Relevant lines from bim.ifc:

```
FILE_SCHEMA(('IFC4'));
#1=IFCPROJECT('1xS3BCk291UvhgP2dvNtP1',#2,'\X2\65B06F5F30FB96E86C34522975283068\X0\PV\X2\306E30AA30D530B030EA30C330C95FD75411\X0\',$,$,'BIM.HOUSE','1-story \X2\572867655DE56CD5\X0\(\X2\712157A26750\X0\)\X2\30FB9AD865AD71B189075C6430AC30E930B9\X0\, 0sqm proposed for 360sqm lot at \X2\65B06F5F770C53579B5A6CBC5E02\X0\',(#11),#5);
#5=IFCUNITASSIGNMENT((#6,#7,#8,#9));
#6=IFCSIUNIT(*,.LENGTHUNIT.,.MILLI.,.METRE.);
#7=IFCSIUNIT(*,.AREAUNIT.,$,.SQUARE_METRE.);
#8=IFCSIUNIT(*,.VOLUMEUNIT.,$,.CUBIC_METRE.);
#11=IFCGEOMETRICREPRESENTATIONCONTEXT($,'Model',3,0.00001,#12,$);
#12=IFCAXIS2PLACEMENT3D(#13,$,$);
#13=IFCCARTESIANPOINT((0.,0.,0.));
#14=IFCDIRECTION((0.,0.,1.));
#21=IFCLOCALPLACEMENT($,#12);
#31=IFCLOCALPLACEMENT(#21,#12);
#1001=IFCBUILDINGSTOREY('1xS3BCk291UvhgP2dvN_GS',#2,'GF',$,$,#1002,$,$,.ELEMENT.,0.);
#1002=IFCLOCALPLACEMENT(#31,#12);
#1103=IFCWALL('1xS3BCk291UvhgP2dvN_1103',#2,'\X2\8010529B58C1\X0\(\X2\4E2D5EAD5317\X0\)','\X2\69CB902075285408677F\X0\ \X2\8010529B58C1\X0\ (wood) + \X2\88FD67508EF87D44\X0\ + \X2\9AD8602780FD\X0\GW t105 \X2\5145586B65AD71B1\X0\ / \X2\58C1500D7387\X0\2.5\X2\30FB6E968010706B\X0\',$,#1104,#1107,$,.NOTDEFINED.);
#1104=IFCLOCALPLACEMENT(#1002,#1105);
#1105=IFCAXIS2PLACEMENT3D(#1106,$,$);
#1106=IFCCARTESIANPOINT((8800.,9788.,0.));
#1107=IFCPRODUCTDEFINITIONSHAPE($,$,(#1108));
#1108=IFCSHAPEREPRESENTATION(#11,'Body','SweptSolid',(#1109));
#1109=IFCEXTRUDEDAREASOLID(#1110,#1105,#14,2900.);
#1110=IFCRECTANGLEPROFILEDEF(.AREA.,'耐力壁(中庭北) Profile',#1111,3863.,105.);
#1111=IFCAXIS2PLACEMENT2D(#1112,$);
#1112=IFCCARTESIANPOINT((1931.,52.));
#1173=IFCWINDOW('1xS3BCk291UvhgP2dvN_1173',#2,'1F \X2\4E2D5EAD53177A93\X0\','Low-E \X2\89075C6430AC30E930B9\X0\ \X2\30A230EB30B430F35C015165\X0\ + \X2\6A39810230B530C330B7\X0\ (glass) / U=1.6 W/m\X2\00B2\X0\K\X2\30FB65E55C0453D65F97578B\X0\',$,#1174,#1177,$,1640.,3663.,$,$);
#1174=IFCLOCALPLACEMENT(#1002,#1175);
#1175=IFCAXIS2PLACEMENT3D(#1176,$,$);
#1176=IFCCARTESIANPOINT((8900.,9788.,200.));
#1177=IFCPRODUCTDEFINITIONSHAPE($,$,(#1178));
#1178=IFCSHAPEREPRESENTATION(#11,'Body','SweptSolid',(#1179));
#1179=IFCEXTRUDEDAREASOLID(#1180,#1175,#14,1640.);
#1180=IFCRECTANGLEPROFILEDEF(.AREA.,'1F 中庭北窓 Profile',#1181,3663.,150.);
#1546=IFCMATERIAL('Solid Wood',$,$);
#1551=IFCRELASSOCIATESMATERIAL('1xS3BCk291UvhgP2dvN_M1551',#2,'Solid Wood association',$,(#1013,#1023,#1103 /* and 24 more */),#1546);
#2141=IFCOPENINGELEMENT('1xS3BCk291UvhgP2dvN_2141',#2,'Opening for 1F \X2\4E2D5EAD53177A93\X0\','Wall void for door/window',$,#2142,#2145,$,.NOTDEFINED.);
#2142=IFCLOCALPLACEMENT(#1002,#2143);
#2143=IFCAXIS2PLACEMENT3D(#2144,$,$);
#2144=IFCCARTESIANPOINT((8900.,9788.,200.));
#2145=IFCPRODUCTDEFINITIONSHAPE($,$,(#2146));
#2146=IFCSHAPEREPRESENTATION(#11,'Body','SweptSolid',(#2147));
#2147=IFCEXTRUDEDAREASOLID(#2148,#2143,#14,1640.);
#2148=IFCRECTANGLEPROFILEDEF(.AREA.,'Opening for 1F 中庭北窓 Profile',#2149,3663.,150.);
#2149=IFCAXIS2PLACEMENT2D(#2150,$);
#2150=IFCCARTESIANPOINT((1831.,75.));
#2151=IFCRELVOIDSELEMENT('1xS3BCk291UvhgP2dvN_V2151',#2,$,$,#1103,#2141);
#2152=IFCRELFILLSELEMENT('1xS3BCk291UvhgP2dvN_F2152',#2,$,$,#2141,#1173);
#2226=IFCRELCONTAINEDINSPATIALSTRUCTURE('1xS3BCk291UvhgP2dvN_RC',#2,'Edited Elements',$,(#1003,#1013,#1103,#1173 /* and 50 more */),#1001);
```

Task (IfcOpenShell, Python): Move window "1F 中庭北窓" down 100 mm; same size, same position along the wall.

```python
import numpy as np
import ifcopenshell
import ifcopenshell.api.geometry
import ifcopenshell.util.placement
import ifcopenshell.util.unit

model = ifcopenshell.open("bim.ifc")
unit_scale = ifcopenshell.util.unit.calculate_unit_scale(model)

window = model.by_guid("1xS3BCk291UvhgP2dvN_1173")
opening = window.FillsVoids[0].RelatingOpeningElement
dz = -100.0

shift = np.array([0.0, 0.0, dz])
# The window is not placed relative to its opening, so move both.
for product in (opening, window):
    matrix = ifcopenshell.util.placement.get_local_placement(product.ObjectPlacement)
    matrix[:3, 3] += shift
    ifcopenshell.api.geometry.edit_object_placement(model, product=product, matrix=matrix, is_si=False)

print(f"moved by {dz * unit_scale:+.3f} m")

model.write("bim_updated.ifc")
```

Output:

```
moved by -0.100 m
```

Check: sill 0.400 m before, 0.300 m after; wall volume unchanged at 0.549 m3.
